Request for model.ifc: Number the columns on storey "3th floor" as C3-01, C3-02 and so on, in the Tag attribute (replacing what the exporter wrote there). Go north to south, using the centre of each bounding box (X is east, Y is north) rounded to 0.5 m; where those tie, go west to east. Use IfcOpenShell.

First a look at what the model holds.

```python
import ifcopenshell
import ifcopenshell.util.element
import ifcopenshell.util.placement

model = ifcopenshell.open("model.ifc")
print(model.schema)
storey = next(s for s in model.by_type("IfcBuildingStorey") if s.Name == "3th floor")
columns = [e for e in ifcopenshell.util.element.get_decomposition(storey) if e.is_a("IfcColumn")]
for e in sorted(columns, key=lambda e: e.id()):
    origin = ifcopenshell.util.placement.get_local_placement(e.ObjectPlacement)[:3, 3]
    print(e.id(), e.Tag, e.Name, origin.round(2) + 0.0, sep=" | ")
```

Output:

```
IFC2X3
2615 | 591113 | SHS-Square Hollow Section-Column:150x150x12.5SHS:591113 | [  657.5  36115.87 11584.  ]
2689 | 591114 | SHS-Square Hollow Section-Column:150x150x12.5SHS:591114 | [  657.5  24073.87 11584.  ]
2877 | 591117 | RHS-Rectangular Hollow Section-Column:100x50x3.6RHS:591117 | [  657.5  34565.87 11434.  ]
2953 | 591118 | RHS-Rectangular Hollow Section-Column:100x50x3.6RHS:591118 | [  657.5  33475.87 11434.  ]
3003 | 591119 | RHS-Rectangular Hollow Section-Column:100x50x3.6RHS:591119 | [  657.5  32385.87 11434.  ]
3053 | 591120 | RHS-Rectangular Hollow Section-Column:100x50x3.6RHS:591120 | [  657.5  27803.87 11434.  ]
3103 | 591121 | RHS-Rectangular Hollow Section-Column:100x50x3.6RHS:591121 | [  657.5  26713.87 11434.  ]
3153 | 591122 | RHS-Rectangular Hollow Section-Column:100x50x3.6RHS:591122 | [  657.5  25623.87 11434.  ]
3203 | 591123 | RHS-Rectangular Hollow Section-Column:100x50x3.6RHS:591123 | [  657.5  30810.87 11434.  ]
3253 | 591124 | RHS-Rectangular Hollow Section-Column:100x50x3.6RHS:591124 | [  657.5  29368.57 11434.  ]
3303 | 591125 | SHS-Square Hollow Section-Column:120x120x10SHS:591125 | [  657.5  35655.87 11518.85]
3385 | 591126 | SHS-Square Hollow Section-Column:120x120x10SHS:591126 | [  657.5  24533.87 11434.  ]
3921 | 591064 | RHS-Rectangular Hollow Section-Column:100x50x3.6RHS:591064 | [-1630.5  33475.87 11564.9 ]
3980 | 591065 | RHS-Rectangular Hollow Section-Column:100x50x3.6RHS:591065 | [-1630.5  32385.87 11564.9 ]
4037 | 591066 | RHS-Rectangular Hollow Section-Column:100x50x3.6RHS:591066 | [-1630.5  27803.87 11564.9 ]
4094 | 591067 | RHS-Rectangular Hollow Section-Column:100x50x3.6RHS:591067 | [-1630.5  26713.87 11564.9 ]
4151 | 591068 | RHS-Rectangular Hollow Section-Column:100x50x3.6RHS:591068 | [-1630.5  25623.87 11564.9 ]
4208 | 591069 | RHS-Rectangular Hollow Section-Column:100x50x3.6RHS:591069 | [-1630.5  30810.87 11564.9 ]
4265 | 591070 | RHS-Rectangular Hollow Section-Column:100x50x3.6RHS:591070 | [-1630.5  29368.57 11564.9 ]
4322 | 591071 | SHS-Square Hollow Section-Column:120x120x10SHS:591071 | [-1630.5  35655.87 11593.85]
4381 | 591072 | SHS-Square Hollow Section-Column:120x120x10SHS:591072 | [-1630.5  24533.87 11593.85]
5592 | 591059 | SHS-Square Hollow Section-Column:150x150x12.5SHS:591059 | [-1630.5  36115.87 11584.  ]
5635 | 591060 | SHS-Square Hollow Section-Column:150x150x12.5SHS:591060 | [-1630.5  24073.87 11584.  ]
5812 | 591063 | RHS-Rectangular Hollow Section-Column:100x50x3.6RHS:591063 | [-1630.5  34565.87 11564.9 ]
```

```python
import ifcopenshell
import ifcopenshell.geom
import ifcopenshell.util.element
import ifcopenshell.util.shape

model = ifcopenshell.open("model.ifc")
settings = ifcopenshell.geom.settings()
settings.set("use-world-coords", True)


def centre(element):
    shape = ifcopenshell.geom.create_shape(settings, element)
    return ifcopenshell.util.shape.get_bbox_centroid(shape.geometry)


storey = next(s for s in model.by_type("IfcBuildingStorey") if s.Name == "3th floor")
columns = [e for e in ifcopenshell.util.element.get_decomposition(storey) if e.is_a("IfcColumn")]

# Insertion points can sit at a corner or the storey origin, so sort by the geometry (in metres).
centres = {e: centre(e) for e in columns}
columns.sort(key=lambda e: (-round(centres[e][1] / 0.5), centres[e][0]))

for i, e in enumerate(columns, start=1):
    number = f"C3-{i:02d}"
    e.Tag = number
    print(e.id(), number)

model.write("model_v2.ifc")
```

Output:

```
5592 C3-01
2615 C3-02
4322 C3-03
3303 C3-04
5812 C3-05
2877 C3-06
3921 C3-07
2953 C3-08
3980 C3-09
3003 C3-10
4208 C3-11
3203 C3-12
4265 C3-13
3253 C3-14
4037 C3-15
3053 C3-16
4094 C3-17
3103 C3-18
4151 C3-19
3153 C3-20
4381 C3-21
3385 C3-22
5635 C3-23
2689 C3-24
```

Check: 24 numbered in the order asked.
